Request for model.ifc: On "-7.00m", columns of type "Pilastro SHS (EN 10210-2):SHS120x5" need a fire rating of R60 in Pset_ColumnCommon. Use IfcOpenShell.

First a look at what the model holds.

```python
import ifcopenshell
import ifcopenshell.util.element

model = ifcopenshell.open("model.ifc")
print(model.schema)
storey = next(s for s in model.by_type("IfcBuildingStorey") if s.Name == "-7.00m")
columns = [e for e in ifcopenshell.util.element.get_decomposition(storey) if e.is_a("IfcColumn")]
seen = {}
for e in columns:
    element_type = ifcopenshell.util.element.get_type(e)
    key = (element_type.Name if element_type != e and element_type else None, ifcopenshell.util.element.get_pset(e, "Pset_ColumnCommon", "FireRating"))
    seen[key] = seen.get(key, 0) + 1
for (name, value), count in sorted(seen.items(), key=str):
    print(count, "x", name, "|", value)
```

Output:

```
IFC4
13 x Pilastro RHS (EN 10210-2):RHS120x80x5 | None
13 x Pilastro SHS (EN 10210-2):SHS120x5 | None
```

```python
import ifcopenshell
import ifcopenshell.api.pset
import ifcopenshell.util.element

model = ifcopenshell.open("model.ifc")

storey = next(s for s in model.by_type("IfcBuildingStorey") if s.Name == "-7.00m")
columns = [e for e in ifcopenshell.util.element.get_decomposition(storey) if e.is_a("IfcColumn")]

count = 0
for e in columns:
    element_type = ifcopenshell.util.element.get_type(e)
    if element_type in (None, e) or element_type.Name != "Pilastro SHS (EN 10210-2):SHS120x5":
        continue
    # add_pset returns the element's existing set when there is one.
    pset = ifcopenshell.api.pset.add_pset(model, product=e, name="Pset_ColumnCommon")
    ifcopenshell.api.pset.edit_pset(model, pset=pset, properties={"FireRating": "R60"})
    count += 1

print(count, "columns updated")

model.write("model-out.ifc")
```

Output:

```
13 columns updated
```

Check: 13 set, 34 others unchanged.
